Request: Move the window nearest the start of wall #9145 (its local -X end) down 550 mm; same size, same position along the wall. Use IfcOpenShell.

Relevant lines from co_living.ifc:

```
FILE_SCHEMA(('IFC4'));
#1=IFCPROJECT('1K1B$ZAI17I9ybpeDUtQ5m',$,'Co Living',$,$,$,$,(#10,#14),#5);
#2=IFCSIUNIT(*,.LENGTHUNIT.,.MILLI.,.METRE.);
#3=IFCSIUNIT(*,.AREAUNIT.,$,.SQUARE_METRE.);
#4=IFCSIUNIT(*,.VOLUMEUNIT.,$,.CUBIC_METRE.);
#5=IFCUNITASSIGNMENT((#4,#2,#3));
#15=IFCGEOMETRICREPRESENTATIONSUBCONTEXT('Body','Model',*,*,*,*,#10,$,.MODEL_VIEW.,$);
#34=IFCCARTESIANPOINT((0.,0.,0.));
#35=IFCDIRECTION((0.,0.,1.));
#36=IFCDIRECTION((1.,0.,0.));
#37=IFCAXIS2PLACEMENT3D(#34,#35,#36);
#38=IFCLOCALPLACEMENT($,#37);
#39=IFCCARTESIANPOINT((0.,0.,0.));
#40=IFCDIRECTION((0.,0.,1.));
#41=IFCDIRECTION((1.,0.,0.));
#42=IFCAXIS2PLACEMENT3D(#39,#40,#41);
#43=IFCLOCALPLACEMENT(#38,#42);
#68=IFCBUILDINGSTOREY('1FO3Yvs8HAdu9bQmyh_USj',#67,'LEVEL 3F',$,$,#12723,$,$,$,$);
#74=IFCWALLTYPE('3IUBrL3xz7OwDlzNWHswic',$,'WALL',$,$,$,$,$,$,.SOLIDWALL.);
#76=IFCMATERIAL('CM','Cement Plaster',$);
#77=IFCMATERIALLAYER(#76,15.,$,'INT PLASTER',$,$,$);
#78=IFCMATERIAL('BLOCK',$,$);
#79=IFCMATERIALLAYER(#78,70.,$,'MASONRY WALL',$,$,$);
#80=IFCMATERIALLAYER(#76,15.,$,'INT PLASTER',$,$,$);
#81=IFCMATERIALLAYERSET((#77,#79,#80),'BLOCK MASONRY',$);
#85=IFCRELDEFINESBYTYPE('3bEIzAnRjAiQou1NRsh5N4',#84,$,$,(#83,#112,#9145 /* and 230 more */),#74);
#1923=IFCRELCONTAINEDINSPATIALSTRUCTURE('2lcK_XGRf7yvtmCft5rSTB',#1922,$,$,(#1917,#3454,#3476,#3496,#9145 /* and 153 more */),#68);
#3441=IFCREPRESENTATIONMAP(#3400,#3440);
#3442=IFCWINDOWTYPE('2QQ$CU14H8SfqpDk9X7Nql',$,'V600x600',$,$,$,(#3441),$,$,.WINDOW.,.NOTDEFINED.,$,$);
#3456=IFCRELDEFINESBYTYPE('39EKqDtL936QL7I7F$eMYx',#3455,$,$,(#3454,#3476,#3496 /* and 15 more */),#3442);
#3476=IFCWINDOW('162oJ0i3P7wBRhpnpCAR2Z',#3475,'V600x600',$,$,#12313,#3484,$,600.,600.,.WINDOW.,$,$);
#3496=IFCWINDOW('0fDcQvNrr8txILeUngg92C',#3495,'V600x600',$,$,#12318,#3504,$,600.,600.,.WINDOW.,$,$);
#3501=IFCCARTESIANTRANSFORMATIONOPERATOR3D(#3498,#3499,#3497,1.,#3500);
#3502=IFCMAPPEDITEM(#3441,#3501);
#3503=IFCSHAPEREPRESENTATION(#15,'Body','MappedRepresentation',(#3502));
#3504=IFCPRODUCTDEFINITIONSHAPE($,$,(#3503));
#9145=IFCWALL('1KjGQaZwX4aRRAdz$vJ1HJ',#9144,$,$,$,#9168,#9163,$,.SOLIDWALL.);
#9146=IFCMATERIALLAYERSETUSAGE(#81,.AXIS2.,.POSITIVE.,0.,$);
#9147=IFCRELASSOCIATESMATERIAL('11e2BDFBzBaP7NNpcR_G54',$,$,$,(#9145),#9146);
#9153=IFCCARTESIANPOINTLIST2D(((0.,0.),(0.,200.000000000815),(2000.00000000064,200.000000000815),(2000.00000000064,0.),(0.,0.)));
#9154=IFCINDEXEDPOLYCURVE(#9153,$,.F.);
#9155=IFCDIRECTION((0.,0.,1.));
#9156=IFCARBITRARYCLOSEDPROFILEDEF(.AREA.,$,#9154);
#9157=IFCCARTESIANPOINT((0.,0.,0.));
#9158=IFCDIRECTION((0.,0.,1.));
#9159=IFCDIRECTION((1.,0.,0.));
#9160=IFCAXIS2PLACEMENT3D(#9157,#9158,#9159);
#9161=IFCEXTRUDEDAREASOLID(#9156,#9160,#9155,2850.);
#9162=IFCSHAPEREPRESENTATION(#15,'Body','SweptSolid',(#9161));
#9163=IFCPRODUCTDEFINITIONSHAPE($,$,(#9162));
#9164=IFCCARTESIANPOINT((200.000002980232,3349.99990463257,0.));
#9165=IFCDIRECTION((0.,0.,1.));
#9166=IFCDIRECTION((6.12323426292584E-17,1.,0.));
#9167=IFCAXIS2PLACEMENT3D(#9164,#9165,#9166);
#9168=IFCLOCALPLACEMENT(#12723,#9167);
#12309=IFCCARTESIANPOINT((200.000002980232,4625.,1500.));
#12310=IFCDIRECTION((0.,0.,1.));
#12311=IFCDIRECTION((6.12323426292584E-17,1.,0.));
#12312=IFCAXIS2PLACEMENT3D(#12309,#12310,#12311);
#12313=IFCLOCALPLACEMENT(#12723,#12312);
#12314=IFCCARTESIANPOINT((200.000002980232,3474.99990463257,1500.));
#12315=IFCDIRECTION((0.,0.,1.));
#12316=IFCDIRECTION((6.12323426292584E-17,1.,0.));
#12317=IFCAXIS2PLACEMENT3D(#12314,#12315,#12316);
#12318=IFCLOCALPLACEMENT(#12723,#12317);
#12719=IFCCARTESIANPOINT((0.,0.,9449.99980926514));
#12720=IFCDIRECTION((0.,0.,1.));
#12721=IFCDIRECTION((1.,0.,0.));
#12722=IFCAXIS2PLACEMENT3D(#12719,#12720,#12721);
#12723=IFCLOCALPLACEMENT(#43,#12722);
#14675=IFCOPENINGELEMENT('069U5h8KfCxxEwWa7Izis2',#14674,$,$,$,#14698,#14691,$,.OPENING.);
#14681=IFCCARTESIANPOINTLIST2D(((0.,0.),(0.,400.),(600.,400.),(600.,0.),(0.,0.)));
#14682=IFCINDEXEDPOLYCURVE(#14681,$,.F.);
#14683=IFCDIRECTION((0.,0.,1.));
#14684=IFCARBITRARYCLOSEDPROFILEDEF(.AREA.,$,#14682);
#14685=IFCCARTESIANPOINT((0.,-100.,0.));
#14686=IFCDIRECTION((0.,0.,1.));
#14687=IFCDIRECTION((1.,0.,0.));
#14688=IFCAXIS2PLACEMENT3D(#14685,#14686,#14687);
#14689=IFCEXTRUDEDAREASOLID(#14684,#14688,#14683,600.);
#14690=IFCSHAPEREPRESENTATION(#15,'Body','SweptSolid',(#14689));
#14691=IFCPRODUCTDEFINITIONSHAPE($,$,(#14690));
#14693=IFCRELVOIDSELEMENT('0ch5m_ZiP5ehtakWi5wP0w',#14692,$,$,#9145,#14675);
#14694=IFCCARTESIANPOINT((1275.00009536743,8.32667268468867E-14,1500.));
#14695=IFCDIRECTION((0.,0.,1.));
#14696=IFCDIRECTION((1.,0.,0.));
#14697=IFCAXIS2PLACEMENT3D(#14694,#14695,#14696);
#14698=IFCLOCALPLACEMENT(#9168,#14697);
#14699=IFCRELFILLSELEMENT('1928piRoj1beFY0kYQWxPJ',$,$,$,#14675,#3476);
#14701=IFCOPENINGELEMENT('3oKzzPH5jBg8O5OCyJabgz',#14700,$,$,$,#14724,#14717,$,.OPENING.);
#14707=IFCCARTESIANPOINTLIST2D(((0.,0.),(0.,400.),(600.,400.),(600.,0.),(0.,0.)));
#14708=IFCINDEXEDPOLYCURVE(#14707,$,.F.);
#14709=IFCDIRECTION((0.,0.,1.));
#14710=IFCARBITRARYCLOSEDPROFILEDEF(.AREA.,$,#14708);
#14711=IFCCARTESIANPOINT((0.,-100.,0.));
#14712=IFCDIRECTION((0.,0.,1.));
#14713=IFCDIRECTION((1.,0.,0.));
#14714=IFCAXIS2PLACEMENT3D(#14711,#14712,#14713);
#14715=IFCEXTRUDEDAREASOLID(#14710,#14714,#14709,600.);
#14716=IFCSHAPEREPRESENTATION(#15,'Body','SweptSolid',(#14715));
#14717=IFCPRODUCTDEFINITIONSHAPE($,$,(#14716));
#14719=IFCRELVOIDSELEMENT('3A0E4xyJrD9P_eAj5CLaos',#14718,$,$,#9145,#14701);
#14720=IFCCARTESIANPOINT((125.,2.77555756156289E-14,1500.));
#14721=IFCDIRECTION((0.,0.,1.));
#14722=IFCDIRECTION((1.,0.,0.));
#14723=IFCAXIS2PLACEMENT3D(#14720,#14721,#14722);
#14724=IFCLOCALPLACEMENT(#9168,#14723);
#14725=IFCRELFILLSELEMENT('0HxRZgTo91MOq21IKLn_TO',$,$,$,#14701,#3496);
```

```python
import numpy as np
import ifcopenshell
import ifcopenshell.api.geometry
import ifcopenshell.util.placement
import ifcopenshell.util.unit

model = ifcopenshell.open("co_living.ifc")
unit_scale = ifcopenshell.util.unit.calculate_unit_scale(model)

window = model.by_id(3496)
opening = window.FillsVoids[0].RelatingOpeningElement
dz = -0.55 / unit_scale

shift = np.array([0.0, 0.0, dz])
# The window is not placed relative to its opening, so move both.
for product in (opening, window):
    matrix = ifcopenshell.util.placement.get_local_placement(product.ObjectPlacement)
    matrix[:3, 3] += shift
    ifcopenshell.api.geometry.edit_object_placement(model, product=product, matrix=matrix, is_si=False)

print(f"moved by {dz * unit_scale:+.3f} m")

model.write("co_living_v2.ifc")
```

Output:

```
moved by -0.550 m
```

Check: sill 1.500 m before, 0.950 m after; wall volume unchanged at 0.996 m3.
